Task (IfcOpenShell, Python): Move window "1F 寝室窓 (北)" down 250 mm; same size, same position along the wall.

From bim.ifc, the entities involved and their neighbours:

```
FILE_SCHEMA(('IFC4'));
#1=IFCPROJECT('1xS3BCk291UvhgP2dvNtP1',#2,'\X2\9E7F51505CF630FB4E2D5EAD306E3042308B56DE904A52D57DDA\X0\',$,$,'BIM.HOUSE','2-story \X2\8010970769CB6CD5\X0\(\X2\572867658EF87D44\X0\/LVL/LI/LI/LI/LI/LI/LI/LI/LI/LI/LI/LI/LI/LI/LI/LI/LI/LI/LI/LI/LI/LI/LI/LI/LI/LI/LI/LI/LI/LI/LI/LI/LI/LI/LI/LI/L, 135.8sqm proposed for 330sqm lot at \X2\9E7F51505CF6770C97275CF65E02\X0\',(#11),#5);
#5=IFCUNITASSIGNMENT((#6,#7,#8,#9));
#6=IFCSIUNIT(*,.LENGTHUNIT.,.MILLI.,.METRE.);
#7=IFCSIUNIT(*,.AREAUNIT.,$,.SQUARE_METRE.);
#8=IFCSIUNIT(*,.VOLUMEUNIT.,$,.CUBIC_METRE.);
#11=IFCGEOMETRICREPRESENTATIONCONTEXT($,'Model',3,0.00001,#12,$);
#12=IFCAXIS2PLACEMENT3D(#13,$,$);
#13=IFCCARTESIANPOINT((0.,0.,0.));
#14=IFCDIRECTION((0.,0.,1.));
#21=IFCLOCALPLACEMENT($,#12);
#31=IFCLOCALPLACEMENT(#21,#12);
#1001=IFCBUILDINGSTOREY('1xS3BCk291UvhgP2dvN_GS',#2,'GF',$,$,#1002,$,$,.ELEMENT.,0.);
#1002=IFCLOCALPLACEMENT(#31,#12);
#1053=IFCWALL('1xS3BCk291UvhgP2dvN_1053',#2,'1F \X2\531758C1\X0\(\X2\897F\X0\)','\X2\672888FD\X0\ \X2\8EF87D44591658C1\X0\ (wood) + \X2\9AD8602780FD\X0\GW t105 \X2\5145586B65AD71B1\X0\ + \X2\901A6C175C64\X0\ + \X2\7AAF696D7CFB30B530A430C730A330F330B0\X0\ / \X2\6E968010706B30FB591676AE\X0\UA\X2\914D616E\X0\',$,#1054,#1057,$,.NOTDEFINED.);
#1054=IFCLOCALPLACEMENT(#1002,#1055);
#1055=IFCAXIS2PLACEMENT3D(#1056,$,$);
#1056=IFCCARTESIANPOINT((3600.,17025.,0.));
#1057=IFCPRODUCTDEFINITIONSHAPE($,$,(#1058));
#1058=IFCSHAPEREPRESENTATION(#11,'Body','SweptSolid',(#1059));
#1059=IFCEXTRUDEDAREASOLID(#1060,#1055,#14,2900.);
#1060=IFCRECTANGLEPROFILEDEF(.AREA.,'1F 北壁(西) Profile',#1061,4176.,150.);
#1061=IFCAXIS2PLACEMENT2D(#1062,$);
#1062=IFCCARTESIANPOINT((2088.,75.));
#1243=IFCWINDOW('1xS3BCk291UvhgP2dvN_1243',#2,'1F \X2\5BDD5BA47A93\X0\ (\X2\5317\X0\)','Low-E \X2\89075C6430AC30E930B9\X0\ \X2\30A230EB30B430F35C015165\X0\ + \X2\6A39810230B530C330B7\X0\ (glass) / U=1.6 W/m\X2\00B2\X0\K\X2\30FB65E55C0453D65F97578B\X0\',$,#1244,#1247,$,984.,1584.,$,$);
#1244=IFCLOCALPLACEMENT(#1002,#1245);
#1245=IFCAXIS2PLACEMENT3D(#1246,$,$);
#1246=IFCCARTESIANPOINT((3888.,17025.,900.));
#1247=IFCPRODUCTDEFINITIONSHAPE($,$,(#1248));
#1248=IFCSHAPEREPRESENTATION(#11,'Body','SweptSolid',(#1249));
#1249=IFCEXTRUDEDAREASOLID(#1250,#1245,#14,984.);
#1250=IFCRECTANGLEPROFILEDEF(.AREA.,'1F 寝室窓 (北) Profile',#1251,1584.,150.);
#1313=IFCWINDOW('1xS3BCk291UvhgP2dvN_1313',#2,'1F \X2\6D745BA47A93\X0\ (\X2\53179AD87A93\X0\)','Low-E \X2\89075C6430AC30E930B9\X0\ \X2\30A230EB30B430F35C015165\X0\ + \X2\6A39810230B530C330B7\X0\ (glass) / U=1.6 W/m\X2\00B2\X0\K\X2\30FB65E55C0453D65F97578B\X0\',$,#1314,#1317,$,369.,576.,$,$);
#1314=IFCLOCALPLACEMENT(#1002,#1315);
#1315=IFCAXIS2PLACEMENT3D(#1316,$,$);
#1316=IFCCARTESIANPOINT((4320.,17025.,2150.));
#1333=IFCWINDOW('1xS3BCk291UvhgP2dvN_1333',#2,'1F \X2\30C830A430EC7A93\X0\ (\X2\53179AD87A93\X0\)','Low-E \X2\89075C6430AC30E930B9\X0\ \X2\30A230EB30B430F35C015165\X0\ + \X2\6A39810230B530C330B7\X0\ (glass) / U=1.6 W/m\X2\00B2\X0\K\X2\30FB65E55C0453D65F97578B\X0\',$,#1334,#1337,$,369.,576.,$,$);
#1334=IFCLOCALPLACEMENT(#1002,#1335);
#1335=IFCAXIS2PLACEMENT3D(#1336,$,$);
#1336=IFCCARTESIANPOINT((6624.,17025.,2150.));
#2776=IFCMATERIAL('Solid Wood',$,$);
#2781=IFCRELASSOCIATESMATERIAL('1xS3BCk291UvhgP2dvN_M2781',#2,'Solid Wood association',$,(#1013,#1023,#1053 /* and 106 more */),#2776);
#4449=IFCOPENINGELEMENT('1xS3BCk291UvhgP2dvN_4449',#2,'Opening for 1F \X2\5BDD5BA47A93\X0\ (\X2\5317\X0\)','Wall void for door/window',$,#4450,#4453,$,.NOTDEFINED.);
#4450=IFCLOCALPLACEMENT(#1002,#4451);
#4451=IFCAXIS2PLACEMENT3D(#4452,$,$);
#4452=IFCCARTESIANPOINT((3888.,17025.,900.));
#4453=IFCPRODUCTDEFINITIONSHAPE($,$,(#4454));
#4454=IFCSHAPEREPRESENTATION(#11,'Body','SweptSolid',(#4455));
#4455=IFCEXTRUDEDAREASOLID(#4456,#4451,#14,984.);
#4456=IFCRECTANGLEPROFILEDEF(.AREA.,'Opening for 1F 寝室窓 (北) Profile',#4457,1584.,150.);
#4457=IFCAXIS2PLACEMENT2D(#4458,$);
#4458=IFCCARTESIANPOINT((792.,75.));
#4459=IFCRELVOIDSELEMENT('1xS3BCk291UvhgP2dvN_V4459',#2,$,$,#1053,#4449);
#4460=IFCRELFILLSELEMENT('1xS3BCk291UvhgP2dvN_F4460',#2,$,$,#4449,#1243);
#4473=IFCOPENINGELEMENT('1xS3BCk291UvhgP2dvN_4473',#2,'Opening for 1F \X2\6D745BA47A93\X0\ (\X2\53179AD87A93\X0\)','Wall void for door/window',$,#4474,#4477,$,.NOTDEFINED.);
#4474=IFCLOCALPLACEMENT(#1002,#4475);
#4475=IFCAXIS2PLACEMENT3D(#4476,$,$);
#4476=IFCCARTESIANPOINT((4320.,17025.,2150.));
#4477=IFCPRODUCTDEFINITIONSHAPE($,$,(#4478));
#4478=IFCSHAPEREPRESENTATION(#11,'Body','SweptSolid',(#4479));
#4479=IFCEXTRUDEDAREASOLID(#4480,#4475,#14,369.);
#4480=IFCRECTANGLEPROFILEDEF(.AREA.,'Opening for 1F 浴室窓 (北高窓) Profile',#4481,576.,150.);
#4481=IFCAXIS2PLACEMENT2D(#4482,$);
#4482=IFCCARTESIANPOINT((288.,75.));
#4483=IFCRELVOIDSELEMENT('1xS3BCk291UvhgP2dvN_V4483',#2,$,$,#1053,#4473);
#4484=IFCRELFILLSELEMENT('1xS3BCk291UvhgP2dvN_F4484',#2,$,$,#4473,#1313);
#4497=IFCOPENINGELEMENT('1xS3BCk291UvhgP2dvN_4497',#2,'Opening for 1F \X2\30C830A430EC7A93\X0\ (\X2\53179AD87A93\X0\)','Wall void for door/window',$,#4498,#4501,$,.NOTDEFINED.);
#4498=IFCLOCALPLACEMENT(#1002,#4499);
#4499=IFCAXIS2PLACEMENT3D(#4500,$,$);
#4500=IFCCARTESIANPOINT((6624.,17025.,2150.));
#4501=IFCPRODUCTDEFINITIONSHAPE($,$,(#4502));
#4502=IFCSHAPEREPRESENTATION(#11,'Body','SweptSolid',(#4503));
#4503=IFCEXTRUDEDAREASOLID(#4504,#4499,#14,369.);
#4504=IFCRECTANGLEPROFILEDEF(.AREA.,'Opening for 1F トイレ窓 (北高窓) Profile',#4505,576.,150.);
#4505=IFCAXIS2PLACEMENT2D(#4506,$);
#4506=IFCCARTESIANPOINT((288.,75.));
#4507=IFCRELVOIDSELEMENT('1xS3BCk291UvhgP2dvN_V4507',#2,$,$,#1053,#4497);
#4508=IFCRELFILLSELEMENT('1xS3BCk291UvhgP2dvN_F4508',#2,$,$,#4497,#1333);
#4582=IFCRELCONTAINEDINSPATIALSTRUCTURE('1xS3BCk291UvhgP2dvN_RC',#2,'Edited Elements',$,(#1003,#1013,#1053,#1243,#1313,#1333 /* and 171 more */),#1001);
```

```python
import numpy as np
import ifcopenshell
import ifcopenshell.api.geometry
import ifcopenshell.util.placement
import ifcopenshell.util.unit

model = ifcopenshell.open("bim.ifc")
unit_scale = ifcopenshell.util.unit.calculate_unit_scale(model)

window = model.by_guid("1xS3BCk291UvhgP2dvN_1243")
opening = window.FillsVoids[0].RelatingOpeningElement
dz = -250.0

shift = np.array([0.0, 0.0, dz])
# The window is not placed relative to its opening, so move both.
for product in (opening, window):
    matrix = ifcopenshell.util.placement.get_local_placement(product.ObjectPlacement)
    matrix[:3, 3] += shift
    ifcopenshell.api.geometry.edit_object_placement(model, product=product, matrix=matrix, is_si=False)

print(f"moved by {dz * unit_scale:+.3f} m")

model.write("bim_v2.ifc")
```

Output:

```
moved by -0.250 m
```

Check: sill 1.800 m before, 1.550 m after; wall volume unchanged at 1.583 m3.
